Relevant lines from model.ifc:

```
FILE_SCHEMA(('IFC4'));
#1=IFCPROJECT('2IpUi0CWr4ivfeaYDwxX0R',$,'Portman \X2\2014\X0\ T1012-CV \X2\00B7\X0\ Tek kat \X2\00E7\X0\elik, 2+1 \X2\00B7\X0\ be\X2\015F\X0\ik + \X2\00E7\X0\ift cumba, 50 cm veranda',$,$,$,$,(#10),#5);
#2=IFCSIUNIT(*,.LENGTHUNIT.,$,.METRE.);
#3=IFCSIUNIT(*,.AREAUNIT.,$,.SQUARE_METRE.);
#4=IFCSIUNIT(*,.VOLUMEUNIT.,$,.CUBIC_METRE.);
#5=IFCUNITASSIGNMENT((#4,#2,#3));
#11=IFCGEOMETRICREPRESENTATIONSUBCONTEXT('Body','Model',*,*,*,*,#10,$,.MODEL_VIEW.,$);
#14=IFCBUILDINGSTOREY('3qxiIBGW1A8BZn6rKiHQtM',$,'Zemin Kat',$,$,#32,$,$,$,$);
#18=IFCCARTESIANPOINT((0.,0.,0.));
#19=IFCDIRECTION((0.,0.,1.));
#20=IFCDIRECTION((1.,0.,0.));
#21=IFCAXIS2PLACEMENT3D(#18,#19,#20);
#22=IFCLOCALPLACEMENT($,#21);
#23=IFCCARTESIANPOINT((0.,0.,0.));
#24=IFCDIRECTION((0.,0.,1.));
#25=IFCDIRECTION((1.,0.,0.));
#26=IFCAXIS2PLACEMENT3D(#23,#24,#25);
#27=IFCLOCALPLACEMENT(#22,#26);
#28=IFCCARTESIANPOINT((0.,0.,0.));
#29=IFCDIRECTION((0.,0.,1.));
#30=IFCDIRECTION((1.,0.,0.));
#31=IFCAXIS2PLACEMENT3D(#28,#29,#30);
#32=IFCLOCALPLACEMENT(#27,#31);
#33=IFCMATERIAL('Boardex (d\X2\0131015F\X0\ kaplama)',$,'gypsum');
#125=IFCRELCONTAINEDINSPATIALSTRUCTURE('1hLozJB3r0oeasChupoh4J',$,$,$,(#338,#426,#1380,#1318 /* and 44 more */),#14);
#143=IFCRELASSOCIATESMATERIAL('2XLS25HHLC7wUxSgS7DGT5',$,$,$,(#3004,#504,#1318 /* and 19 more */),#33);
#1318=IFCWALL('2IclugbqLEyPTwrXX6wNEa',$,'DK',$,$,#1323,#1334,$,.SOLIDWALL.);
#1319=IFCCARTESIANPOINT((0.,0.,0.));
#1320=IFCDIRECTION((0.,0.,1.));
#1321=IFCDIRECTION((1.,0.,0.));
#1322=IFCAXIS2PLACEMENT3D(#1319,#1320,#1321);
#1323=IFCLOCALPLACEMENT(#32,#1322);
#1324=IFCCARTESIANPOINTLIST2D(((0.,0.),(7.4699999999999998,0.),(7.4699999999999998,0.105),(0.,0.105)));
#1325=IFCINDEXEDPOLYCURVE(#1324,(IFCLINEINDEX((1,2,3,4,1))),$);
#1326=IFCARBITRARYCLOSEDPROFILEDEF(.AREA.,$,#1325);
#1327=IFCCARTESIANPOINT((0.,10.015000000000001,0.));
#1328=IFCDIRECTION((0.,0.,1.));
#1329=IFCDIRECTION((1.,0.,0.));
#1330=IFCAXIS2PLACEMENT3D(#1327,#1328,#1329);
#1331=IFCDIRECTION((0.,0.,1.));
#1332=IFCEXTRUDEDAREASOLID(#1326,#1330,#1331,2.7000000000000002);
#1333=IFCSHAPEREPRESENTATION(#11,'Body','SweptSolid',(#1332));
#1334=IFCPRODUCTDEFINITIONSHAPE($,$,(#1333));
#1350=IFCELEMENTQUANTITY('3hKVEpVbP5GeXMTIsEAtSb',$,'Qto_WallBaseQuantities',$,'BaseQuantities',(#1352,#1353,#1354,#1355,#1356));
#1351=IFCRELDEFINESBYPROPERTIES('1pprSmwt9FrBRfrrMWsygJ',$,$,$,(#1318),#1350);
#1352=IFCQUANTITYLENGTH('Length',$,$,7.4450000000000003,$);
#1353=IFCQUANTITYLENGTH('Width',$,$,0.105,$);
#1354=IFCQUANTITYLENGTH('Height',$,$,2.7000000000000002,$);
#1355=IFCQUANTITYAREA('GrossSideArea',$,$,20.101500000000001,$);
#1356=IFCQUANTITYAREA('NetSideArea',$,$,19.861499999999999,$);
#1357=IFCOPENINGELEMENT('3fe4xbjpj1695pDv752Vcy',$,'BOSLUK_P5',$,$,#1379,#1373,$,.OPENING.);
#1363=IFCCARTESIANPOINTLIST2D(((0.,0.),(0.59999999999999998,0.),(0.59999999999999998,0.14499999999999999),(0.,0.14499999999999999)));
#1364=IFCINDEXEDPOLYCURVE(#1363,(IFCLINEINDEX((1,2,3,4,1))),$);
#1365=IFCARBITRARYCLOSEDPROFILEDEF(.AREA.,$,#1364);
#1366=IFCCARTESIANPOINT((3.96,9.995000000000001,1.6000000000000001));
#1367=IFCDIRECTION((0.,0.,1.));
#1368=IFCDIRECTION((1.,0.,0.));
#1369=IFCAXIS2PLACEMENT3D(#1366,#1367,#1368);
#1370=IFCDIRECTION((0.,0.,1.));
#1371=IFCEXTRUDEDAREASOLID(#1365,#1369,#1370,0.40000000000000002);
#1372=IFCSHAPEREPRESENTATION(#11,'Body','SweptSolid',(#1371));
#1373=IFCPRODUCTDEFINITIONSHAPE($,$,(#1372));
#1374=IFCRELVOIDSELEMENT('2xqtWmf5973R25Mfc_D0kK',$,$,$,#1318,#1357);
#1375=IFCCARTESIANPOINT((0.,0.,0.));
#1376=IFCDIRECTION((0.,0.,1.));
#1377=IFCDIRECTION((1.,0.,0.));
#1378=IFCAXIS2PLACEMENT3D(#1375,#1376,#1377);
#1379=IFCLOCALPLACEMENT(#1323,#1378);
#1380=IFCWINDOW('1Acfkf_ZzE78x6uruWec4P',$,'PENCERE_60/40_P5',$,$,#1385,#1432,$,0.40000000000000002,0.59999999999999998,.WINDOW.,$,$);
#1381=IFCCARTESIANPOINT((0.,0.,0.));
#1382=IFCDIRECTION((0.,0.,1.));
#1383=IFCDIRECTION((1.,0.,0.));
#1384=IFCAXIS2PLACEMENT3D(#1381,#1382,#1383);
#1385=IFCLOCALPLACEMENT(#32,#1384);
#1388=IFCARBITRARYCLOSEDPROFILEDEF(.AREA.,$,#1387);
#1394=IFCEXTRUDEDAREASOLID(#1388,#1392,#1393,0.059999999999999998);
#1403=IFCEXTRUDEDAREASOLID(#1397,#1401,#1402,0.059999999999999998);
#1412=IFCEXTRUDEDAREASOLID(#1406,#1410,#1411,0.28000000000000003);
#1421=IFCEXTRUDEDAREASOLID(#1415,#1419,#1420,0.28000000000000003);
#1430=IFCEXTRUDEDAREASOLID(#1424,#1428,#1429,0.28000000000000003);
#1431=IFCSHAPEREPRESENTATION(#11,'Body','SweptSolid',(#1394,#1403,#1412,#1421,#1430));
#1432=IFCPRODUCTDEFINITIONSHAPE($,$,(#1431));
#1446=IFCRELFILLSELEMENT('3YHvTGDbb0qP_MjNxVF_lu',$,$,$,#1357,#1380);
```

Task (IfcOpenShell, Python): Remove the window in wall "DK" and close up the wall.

```python
import ifcopenshell
import ifcopenshell.api.feature
import ifcopenshell.api.pset
import ifcopenshell.api.root
import ifcopenshell.geom
import ifcopenshell.util.element
import ifcopenshell.util.shape
import ifcopenshell.util.unit

model = ifcopenshell.open("model.ifc")
area_scale = ifcopenshell.util.unit.calculate_unit_scale(model, "AREAUNIT")
settings = ifcopenshell.geom.settings()


def volume(element):
    """Net volume in cubic metres, openings subtracted."""
    shape = ifcopenshell.geom.create_shape(settings, element)
    return ifcopenshell.util.shape.get_volume(shape.geometry)


window = model.by_guid("1Acfkf_ZzE78x6uruWec4P")
opening = window.FillsVoids[0].RelatingOpeningElement
wall = opening.VoidsElements[0].RelatingBuildingElement
before = volume(wall)

ifcopenshell.api.root.remove_product(model, product=window)
ifcopenshell.api.feature.remove_feature(model, feature=opening)

after = volume(wall)
thickness = 0.105  # wall thickness in metres

# Update the wall's stored quantities.
qto = model.by_id(ifcopenshell.util.element.get_pset(wall, "Qto_WallBaseQuantities", should_inherit=False)["id"])
ifcopenshell.api.pset.edit_qto(model, qto=qto, properties={"NetSideArea": after / thickness / area_scale})

print(f"wall volume {before:.3f} -> {after:.3f} m3")

model.write("model_v2.ifc")
```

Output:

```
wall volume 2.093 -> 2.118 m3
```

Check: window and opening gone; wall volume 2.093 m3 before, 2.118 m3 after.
